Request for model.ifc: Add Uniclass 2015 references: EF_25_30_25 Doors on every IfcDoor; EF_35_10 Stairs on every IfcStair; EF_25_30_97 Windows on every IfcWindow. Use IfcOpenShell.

First a look at what the model holds.

```python
import ifcopenshell

model = ifcopenshell.open("model.ifc")
print(model.schema)
print("classifications:", [c.Name for c in model.by_type("IfcClassification")])
for ifc_class in ("IfcDoor", "IfcRoof", "IfcStair", "IfcWall", "IfcWindow"):
    print(ifc_class, len(model.by_type(ifc_class)))
```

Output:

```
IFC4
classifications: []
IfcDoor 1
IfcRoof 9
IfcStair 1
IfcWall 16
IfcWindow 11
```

```python
import ifcopenshell
import ifcopenshell.api.classification

model = ifcopenshell.open("model.ifc")

system = ifcopenshell.api.classification.add_classification(model, classification="Uniclass 2015")

codes = {
    "IfcDoor": ("EF_25_30_25", "Doors"),
    "IfcStair": ("EF_35_10", "Stairs"),
    "IfcWindow": ("EF_25_30_97", "Windows"),
}
for ifc_class, (code, name) in codes.items():
    products = model.by_type(ifc_class)
    ifcopenshell.api.classification.add_reference(
        model, products=products, classification=system, identification=code, name=name
    )
    print(code, len(products))

model.write("model_v2.ifc")
```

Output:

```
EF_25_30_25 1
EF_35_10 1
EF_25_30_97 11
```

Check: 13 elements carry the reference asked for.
